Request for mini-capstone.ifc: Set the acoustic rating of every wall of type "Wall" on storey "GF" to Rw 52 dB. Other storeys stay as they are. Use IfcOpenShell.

First a look at what the model holds.

```python
import ifcopenshell
import ifcopenshell.util.element

model = ifcopenshell.open("mini-capstone.ifc")
print(model.schema)
storey = next(s for s in model.by_type("IfcBuildingStorey") if s.Name == "GF")
walls = [e for e in ifcopenshell.util.element.get_decomposition(storey) if e.is_a("IfcWall")]
seen = {}
for e in walls:
    element_type = ifcopenshell.util.element.get_type(e)
    key = (element_type.Name if element_type != e and element_type else None, ifcopenshell.util.element.get_pset(e, "Pset_WallCommon", "AcousticRating"))
    seen[key] = seen.get(key, 0) + 1
for (name, value), count in sorted(seen.items(), key=str):
    print(count, "x", name, "|", value)
```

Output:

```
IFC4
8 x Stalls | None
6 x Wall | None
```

```python
import ifcopenshell
import ifcopenshell.api.pset
import ifcopenshell.util.element

model = ifcopenshell.open("mini-capstone.ifc")

storey = next(s for s in model.by_type("IfcBuildingStorey") if s.Name == "GF")
walls = [e for e in ifcopenshell.util.element.get_decomposition(storey) if e.is_a("IfcWall")]

count = 0
for e in walls:
    element_type = ifcopenshell.util.element.get_type(e)
    if element_type in (None, e) or element_type.Name != "Wall":
        continue
    # add_pset returns the element's existing set when there is one.
    pset = ifcopenshell.api.pset.add_pset(model, product=e, name="Pset_WallCommon")
    ifcopenshell.api.pset.edit_pset(model, pset=pset, properties={"AcousticRating": "Rw 52 dB"})
    count += 1

print(count, "walls updated")

model.write("mini-capstone_edited.ifc")
```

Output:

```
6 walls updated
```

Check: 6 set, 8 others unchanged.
